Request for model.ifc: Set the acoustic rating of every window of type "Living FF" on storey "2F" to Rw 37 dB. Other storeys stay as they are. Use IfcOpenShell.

First a look at what the model holds.

```python
import ifcopenshell
import ifcopenshell.util.element

model = ifcopenshell.open("model.ifc")
print(model.schema)
storey = next(s for s in model.by_type("IfcBuildingStorey") if s.Name == "2F")
windows = [e for e in ifcopenshell.util.element.get_decomposition(storey) if e.is_a("IfcWindow")]
seen = {}
for e in windows:
    element_type = ifcopenshell.util.element.get_type(e)
    key = (element_type.Name if element_type != e and element_type else None, ifcopenshell.util.element.get_pset(e, "Pset_WindowCommon", "AcousticRating"))
    seen[key] = seen.get(key, 0) + 1
for (name, value), count in sorted(seen.items(), key=str):
    print(count, "x", name, "|", value)
```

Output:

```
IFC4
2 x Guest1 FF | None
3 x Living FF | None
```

```python
import ifcopenshell
import ifcopenshell.api.pset
import ifcopenshell.util.element

model = ifcopenshell.open("model.ifc")

storey = next(s for s in model.by_type("IfcBuildingStorey") if s.Name == "2F")
windows = [e for e in ifcopenshell.util.element.get_decomposition(storey) if e.is_a("IfcWindow")]

count = 0
for e in windows:
    element_type = ifcopenshell.util.element.get_type(e)
    if element_type in (None, e) or element_type.Name != "Living FF":
        continue
    # add_pset returns the element's existing set when there is one.
    pset = ifcopenshell.api.pset.add_pset(model, product=e, name="Pset_WindowCommon")
    ifcopenshell.api.pset.edit_pset(model, pset=pset, properties={"AcousticRating": "Rw 37 dB"})
    count += 1

print(count, "windows updated")

model.write("model_v2.ifc")
```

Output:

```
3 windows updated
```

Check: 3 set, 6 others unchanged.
